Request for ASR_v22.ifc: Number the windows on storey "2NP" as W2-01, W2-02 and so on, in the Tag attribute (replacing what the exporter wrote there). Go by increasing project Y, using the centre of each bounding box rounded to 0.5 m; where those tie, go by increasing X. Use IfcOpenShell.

First a look at what the model holds.

```python
import ifcopenshell
import ifcopenshell.util.element
import ifcopenshell.util.placement

model = ifcopenshell.open("ASR_v22.ifc")
print(model.schema)
storey = next(s for s in model.by_type("IfcBuildingStorey") if s.Name == "2NP")
windows = [e for e in ifcopenshell.util.element.get_decomposition(storey) if e.is_a("IfcWindow")]
for e in sorted(windows, key=lambda e: e.id()):
    origin = ifcopenshell.util.placement.get_local_placement(e.ObjectPlacement)[:3, 3]
    print(e.id(), e.Tag, e.Name, origin.round(2) + 0.0, sep=" | ")
```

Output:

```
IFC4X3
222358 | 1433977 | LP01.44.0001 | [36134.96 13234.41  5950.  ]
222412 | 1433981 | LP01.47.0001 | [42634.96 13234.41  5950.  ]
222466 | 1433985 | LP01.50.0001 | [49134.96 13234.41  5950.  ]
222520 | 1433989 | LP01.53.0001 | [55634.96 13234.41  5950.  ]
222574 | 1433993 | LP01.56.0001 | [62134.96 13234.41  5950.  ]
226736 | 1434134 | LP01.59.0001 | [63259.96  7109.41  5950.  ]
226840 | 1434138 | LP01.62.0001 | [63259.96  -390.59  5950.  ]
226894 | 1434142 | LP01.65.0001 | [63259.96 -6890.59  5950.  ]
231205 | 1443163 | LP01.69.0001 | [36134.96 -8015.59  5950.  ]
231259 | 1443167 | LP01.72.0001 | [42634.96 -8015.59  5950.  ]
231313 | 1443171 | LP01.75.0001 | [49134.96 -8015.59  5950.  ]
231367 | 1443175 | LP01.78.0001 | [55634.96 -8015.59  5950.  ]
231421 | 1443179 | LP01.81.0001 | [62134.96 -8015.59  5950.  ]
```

```python
import ifcopenshell
import ifcopenshell.geom
import ifcopenshell.util.element
import ifcopenshell.util.shape

model = ifcopenshell.open("ASR_v22.ifc")
settings = ifcopenshell.geom.settings()
settings.set("use-world-coords", True)


def centre(element):
    shape = ifcopenshell.geom.create_shape(settings, element)
    return ifcopenshell.util.shape.get_bbox_centroid(shape.geometry)


storey = next(s for s in model.by_type("IfcBuildingStorey") if s.Name == "2NP")
windows = [e for e in ifcopenshell.util.element.get_decomposition(storey) if e.is_a("IfcWindow")]

# Insertion points can sit at a corner or the storey origin, so sort by the geometry (in metres).
centres = {e: centre(e) for e in windows}
windows.sort(key=lambda e: (round(centres[e][1] / 0.5), centres[e][0]))

for i, e in enumerate(windows, start=1):
    number = f"W2-{i:02d}"
    e.Tag = number
    print(e.id(), number)

model.write("ASR_v22_updated.ifc")
```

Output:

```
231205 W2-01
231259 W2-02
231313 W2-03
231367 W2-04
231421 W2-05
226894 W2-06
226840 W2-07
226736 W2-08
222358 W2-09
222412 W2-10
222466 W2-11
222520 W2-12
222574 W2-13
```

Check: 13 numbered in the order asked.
